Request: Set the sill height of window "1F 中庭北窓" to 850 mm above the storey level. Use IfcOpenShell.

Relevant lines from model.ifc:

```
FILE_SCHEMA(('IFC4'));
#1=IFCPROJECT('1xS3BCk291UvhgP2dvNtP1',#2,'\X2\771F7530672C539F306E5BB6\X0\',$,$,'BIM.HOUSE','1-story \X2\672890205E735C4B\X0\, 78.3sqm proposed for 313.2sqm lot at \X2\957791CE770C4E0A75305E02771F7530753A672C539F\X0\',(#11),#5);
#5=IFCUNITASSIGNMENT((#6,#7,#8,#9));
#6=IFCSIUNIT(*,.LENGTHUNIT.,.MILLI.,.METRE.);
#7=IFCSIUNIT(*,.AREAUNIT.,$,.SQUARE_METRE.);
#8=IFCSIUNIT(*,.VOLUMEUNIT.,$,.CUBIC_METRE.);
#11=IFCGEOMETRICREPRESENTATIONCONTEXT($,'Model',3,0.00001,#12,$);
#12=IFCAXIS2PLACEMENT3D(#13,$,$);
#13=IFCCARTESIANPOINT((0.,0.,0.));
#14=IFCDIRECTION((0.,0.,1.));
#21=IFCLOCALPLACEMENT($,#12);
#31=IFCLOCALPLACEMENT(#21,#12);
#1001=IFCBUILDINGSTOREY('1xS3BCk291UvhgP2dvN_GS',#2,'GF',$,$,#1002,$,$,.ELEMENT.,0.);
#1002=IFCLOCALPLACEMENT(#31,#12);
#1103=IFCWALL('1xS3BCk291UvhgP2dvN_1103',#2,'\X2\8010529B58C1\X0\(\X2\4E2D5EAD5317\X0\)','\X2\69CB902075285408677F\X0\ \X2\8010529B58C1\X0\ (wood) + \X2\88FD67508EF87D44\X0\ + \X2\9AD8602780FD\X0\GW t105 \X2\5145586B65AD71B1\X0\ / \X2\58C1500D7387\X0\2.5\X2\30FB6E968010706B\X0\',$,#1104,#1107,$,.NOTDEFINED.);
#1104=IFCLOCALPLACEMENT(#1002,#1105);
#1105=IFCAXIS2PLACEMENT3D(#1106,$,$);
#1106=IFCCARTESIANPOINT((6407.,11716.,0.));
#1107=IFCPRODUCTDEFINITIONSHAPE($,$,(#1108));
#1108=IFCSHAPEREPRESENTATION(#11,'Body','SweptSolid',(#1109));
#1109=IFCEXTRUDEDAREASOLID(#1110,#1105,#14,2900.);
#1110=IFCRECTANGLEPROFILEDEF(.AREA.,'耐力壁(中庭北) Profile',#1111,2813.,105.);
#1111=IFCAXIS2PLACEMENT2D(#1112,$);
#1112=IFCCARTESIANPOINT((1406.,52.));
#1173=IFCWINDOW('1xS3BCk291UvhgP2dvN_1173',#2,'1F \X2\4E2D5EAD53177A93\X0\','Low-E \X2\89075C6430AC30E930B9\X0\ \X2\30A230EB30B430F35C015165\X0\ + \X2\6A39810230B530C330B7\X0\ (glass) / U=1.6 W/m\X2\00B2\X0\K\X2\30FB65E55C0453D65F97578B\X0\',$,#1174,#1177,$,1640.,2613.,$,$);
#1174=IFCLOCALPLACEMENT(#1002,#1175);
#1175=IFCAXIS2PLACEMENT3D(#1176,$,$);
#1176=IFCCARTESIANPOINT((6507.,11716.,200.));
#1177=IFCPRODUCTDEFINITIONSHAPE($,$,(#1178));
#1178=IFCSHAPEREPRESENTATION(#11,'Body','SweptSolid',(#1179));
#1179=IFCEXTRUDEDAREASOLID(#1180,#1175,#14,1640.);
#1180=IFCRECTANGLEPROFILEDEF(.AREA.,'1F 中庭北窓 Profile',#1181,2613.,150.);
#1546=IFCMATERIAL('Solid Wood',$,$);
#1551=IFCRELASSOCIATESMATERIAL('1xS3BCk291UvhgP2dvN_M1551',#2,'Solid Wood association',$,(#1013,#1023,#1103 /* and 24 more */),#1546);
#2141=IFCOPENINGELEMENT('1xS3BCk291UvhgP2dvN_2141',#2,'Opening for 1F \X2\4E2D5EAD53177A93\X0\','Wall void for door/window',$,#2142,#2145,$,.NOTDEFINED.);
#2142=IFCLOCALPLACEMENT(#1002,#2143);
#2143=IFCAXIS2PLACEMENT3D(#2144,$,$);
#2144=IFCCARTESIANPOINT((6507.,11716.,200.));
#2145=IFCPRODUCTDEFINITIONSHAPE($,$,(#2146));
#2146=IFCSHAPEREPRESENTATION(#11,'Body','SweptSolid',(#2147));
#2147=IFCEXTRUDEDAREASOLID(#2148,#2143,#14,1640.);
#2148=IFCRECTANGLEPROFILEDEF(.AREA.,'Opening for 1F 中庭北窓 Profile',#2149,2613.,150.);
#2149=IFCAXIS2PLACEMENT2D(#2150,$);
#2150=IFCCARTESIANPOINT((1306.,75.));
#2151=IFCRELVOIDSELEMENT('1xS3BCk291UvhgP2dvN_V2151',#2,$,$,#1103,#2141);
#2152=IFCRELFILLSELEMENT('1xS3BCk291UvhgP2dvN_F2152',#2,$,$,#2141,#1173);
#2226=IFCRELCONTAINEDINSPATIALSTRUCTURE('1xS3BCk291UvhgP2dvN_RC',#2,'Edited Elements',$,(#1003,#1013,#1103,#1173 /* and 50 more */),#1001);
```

```python
import numpy as np
import ifcopenshell
import ifcopenshell.api.geometry
import ifcopenshell.geom
import ifcopenshell.util.element
import ifcopenshell.util.placement
import ifcopenshell.util.shape
import ifcopenshell.util.unit

model = ifcopenshell.open("model.ifc")
unit_scale = ifcopenshell.util.unit.calculate_unit_scale(model)

window = model.by_id(1173)
opening = window.FillsVoids[0].RelatingOpeningElement
storey = ifcopenshell.util.element.get_container(window, ifc_class="IfcBuildingStorey")
level = ifcopenshell.util.placement.get_local_placement(storey.ObjectPlacement)[2, 3]

# The opening's origin need not be at the sill, so measure its lowest point.
shape = ifcopenshell.geom.create_shape(ifcopenshell.geom.settings(), opening)
bottom = ifcopenshell.util.shape.get_shape_bottom_elevation(shape, shape.geometry) / unit_scale
dz = level + 0.85 / unit_scale - bottom

shift = np.array([0.0, 0.0, dz])
# The window is not placed relative to its opening, so move both.
for product in (opening, window):
    matrix = ifcopenshell.util.placement.get_local_placement(product.ObjectPlacement)
    matrix[:3, 3] += shift
    ifcopenshell.api.geometry.edit_object_placement(model, product=product, matrix=matrix, is_si=False)

print(f"moved by {dz * unit_scale:+.3f} m")

model.write("model_rev.ifc")
```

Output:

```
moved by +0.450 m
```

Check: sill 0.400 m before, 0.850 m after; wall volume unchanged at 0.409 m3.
